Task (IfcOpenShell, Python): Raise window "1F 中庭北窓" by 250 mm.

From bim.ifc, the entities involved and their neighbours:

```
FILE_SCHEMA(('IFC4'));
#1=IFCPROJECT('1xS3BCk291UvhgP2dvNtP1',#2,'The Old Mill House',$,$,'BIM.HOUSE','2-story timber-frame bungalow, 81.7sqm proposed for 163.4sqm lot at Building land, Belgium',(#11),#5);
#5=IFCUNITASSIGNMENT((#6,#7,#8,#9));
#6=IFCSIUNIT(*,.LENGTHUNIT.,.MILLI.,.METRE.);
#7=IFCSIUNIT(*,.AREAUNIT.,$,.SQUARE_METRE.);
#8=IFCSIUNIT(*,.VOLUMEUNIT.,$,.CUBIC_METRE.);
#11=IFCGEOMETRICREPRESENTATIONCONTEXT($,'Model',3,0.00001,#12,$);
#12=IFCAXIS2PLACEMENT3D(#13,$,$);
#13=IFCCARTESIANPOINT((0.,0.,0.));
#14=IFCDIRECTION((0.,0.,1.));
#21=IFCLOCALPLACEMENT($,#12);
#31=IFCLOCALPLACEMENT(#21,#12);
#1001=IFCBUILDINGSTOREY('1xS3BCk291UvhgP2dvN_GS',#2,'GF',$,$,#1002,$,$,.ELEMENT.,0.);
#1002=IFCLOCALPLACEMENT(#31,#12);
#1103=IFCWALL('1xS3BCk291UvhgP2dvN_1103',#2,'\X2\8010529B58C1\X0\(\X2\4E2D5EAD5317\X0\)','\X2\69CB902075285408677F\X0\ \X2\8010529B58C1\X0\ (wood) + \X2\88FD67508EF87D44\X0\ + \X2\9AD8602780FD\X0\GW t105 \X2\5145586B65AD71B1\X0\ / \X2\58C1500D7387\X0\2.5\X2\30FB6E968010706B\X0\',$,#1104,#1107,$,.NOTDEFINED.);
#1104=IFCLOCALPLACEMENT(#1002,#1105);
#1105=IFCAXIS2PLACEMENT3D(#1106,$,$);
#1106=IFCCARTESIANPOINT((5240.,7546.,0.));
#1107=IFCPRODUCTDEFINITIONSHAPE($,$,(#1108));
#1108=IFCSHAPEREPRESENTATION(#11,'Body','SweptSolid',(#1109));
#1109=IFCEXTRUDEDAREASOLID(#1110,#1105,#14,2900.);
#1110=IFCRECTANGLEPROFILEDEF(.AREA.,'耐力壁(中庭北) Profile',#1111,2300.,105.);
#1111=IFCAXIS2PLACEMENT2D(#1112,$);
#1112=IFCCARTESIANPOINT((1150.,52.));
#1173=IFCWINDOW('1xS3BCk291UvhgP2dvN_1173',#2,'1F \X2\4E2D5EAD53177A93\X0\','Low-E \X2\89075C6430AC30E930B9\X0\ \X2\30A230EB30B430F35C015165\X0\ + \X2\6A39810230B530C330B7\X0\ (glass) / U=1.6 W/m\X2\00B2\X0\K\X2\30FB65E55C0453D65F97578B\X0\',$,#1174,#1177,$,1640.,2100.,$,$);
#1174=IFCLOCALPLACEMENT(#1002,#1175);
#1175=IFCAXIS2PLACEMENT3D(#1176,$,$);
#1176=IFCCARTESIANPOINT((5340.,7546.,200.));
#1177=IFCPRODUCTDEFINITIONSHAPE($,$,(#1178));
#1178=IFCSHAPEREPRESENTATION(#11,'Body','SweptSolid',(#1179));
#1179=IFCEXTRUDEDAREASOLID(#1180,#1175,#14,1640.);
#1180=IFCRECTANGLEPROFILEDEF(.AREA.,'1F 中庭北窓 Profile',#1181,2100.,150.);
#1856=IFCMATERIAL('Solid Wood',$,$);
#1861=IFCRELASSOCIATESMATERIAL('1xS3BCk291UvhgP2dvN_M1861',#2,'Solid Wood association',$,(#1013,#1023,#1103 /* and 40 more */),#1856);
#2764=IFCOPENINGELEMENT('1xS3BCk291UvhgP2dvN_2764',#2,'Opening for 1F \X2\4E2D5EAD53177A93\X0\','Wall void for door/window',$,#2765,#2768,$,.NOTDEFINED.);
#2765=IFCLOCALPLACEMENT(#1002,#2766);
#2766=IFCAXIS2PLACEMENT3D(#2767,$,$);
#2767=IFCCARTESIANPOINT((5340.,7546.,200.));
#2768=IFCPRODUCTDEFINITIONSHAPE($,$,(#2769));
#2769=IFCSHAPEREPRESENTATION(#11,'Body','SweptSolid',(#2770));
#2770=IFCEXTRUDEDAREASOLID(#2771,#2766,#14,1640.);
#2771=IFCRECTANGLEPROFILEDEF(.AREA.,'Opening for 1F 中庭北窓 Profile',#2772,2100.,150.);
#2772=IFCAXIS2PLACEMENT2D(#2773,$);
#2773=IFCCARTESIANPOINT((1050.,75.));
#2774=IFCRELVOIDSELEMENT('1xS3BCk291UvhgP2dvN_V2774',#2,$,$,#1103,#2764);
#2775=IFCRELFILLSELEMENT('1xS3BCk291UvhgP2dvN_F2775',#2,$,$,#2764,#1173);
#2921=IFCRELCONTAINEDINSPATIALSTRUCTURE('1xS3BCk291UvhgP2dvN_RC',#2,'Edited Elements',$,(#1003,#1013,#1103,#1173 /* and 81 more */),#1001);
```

```python
import numpy as np
import ifcopenshell
import ifcopenshell.api.geometry
import ifcopenshell.util.placement
import ifcopenshell.util.unit

model = ifcopenshell.open("bim.ifc")
unit_scale = ifcopenshell.util.unit.calculate_unit_scale(model)

window = model.by_guid("1xS3BCk291UvhgP2dvN_1173")
opening = window.FillsVoids[0].RelatingOpeningElement
dz = 0.25 / unit_scale

shift = np.array([0.0, 0.0, dz])
# The window is not placed relative to its opening, so move both.
for product in (opening, window):
    matrix = ifcopenshell.util.placement.get_local_placement(product.ObjectPlacement)
    matrix[:3, 3] += shift
    ifcopenshell.api.geometry.edit_object_placement(model, product=product, matrix=matrix, is_si=False)

print(f"moved by {dz * unit_scale:+.3f} m")

model.write("bim_updated.ifc")
```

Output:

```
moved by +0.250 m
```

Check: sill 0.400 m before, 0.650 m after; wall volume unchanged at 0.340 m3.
